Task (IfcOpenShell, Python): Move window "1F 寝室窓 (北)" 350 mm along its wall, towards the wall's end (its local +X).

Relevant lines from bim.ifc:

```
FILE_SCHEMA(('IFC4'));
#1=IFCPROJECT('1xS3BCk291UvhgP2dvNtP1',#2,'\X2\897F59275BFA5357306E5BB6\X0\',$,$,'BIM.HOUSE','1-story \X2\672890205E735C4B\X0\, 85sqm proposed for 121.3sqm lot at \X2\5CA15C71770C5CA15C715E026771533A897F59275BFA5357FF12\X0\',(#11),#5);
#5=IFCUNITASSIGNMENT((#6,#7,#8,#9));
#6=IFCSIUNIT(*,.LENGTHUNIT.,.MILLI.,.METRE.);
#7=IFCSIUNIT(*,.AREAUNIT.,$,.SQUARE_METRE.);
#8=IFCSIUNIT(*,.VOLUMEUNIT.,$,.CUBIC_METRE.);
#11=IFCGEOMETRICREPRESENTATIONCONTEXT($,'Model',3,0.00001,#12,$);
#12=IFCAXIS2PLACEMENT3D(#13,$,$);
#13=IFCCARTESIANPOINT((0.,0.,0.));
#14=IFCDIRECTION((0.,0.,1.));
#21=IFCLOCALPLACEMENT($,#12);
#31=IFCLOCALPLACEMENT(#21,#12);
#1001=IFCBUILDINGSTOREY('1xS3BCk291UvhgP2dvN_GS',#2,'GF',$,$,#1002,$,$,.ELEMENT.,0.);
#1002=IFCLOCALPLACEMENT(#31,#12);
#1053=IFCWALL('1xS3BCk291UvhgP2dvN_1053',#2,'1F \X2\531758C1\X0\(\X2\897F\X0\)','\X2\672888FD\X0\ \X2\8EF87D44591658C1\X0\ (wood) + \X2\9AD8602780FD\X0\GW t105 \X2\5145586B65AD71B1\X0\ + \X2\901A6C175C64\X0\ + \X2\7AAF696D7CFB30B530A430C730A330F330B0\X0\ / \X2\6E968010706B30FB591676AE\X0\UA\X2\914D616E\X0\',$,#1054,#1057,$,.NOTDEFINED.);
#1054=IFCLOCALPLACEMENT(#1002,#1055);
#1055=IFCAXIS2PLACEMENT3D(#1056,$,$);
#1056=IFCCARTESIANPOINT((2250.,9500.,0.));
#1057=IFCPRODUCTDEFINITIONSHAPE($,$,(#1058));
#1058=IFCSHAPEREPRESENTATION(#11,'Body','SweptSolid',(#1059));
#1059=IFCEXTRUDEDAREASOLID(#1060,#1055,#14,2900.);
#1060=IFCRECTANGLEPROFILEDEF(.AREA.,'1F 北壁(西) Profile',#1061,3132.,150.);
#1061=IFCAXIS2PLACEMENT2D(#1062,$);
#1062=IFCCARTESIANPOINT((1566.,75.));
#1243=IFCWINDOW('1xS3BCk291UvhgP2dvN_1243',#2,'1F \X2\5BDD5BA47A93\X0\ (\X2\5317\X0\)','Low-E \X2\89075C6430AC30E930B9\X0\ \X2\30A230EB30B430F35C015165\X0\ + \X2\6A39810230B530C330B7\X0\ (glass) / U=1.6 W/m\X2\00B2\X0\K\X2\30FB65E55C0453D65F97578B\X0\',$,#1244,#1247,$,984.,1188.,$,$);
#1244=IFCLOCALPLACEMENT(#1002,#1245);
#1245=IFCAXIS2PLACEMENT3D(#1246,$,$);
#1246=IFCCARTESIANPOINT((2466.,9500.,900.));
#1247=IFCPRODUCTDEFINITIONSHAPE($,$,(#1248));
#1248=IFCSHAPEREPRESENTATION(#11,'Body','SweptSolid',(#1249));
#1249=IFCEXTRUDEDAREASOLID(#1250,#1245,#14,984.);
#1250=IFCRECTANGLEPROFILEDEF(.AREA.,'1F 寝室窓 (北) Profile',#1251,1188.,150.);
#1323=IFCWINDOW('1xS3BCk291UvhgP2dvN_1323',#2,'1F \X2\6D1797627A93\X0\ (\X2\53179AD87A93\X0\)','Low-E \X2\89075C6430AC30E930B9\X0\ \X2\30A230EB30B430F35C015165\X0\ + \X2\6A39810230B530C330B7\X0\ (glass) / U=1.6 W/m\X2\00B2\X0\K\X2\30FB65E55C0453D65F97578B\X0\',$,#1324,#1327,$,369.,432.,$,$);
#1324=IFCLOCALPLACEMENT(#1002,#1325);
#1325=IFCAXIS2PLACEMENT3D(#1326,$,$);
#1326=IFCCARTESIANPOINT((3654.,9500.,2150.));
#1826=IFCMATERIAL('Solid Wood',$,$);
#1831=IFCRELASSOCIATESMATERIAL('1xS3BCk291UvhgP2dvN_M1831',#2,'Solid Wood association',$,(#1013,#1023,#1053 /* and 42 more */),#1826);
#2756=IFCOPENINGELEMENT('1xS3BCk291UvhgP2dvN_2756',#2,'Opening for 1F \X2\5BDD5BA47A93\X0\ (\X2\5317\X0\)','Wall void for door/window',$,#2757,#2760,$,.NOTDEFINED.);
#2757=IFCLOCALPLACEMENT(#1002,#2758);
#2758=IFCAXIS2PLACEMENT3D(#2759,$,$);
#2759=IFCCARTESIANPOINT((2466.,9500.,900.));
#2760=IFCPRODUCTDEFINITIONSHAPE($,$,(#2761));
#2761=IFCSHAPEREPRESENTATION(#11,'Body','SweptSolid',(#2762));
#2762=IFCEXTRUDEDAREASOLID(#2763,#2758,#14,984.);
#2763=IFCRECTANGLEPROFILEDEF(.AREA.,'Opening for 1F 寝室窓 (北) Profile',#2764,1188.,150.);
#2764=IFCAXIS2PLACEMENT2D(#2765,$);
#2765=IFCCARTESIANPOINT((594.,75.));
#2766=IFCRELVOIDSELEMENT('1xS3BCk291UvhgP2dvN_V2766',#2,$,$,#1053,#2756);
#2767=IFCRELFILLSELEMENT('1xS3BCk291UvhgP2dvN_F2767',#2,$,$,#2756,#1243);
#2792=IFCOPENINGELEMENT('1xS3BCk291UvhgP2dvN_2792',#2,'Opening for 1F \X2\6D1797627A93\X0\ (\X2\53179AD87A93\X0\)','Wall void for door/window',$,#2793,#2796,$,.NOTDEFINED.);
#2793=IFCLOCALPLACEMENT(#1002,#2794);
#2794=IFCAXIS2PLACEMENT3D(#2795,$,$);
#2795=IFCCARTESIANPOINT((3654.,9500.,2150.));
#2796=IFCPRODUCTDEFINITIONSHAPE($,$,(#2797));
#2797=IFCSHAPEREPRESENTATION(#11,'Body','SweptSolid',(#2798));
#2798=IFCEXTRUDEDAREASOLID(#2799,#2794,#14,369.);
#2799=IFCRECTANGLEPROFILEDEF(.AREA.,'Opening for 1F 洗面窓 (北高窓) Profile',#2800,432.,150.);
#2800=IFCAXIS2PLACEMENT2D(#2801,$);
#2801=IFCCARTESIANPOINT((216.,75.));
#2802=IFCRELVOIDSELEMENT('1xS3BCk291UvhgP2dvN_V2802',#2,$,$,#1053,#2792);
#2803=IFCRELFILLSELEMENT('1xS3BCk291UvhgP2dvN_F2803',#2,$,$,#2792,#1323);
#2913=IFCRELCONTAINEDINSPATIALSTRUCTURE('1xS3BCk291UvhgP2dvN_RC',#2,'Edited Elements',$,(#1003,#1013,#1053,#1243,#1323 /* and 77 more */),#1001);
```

```python
import ifcopenshell
import ifcopenshell.api.geometry
import ifcopenshell.util.placement
import ifcopenshell.util.unit

model = ifcopenshell.open("bim.ifc")
unit_scale = ifcopenshell.util.unit.calculate_unit_scale(model)

window = model.by_guid("1xS3BCk291UvhgP2dvN_1243")
opening = window.FillsVoids[0].RelatingOpeningElement
wall = opening.VoidsElements[0].RelatingBuildingElement

wall_matrix = ifcopenshell.util.placement.get_local_placement(wall.ObjectPlacement)
shift = wall_matrix[:3, 0] * 0.35 / unit_scale
before = ifcopenshell.util.placement.get_local_placement(window.ObjectPlacement)[:3, 3].copy()

# The window is not placed relative to its opening, so move both.
for product in (opening, window):
    matrix = ifcopenshell.util.placement.get_local_placement(product.ObjectPlacement)
    matrix[:3, 3] += shift
    ifcopenshell.api.geometry.edit_object_placement(model, product=product, matrix=matrix, is_si=False)

after = ifcopenshell.util.placement.get_local_placement(window.ObjectPlacement)[:3, 3]
print("window moved by", (after - before).round(3) + 0.0)

model.write("bim_v2.ifc")
```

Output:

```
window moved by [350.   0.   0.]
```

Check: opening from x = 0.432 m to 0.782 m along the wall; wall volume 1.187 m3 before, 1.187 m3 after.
